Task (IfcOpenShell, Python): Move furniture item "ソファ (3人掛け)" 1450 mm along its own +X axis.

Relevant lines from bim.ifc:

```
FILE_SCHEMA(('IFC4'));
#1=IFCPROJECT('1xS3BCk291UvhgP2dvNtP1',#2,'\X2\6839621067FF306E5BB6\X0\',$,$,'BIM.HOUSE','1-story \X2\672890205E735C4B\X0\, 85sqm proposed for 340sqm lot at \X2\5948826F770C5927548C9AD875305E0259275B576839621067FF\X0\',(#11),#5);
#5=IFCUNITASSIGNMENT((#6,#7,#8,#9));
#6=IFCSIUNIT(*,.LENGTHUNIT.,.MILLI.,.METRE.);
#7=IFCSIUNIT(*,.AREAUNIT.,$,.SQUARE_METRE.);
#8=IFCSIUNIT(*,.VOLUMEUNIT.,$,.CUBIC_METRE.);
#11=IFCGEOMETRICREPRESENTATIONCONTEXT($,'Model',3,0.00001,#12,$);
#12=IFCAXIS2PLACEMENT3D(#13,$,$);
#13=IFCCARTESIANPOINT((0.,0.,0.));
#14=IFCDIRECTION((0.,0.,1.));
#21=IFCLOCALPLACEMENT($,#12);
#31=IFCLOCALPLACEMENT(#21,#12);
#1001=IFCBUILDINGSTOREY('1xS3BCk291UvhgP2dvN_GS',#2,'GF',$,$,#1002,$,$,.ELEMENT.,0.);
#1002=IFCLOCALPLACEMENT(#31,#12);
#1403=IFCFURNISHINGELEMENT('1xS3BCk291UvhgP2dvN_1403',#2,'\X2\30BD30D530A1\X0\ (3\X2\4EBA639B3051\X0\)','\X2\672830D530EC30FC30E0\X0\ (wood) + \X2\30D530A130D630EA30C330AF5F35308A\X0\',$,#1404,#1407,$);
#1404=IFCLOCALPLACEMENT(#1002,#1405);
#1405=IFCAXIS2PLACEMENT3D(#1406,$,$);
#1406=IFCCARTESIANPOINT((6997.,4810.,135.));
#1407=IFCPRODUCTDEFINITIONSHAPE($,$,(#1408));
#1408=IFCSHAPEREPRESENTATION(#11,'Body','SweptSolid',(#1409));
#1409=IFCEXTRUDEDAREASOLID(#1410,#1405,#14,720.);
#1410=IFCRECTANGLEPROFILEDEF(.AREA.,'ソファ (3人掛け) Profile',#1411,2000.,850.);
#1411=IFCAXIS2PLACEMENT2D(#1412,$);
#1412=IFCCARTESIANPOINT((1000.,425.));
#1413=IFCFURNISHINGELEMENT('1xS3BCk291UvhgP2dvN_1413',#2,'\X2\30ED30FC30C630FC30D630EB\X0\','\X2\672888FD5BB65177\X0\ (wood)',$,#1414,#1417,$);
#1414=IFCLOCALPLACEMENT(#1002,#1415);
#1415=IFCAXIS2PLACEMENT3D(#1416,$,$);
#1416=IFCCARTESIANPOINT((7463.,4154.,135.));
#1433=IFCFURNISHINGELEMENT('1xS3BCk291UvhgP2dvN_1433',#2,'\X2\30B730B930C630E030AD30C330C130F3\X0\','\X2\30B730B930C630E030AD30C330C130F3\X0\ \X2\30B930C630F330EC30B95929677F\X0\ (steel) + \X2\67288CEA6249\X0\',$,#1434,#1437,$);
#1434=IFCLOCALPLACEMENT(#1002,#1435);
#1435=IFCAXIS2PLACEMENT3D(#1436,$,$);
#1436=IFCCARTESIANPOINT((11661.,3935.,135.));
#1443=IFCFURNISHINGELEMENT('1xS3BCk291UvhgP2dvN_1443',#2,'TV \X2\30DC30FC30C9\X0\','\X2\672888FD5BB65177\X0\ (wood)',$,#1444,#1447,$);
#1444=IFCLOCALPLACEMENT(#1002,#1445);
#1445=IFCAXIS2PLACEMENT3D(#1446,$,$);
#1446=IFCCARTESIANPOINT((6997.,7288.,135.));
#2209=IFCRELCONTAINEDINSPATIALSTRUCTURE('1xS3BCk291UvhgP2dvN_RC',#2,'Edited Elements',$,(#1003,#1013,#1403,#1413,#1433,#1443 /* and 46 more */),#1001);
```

```python
import ifcopenshell
import ifcopenshell.api.geometry
import ifcopenshell.util.placement

model = ifcopenshell.open("bim.ifc")

item = model.by_guid("1xS3BCk291UvhgP2dvN_1403")
matrix = ifcopenshell.util.placement.get_local_placement(item.ObjectPlacement)
matrix[:3, 3] += matrix[:3, 0] * 1450.0
ifcopenshell.api.geometry.edit_object_placement(model, product=item, matrix=matrix, is_si=False)

print(ifcopenshell.util.placement.get_local_placement(item.ObjectPlacement).round(3) + 0.0)

model.write("bim_edited.ifc")
```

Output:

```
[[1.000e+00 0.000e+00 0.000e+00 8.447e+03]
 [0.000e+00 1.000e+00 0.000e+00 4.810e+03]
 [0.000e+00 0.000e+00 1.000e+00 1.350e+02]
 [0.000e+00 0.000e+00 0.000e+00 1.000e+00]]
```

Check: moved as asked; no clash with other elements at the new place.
